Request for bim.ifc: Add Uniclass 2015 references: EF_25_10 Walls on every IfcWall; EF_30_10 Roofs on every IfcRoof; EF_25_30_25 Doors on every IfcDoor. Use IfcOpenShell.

First a look at what the model holds.

```python
import ifcopenshell

model = ifcopenshell.open("bim.ifc")
print(model.schema)
print("classifications:", [c.Name for c in model.by_type("IfcClassification")])
for ifc_class in ("IfcDoor", "IfcRoof", "IfcStair", "IfcWall", "IfcWindow"):
    print(ifc_class, len(model.by_type(ifc_class)))
```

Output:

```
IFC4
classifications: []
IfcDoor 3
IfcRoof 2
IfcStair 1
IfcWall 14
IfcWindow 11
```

```python
import ifcopenshell
import ifcopenshell.api.classification

model = ifcopenshell.open("bim.ifc")

system = ifcopenshell.api.classification.add_classification(model, classification="Uniclass 2015")

codes = {
    "IfcWall": ("EF_25_10", "Walls"),
    "IfcRoof": ("EF_30_10", "Roofs"),
    "IfcDoor": ("EF_25_30_25", "Doors"),
}
for ifc_class, (code, name) in codes.items():
    products = model.by_type(ifc_class)
    ifcopenshell.api.classification.add_reference(
        model, products=products, classification=system, identification=code, name=name
    )
    print(code, len(products))

model.write("bim-out.ifc")
```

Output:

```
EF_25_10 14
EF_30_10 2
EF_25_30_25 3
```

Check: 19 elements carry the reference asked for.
